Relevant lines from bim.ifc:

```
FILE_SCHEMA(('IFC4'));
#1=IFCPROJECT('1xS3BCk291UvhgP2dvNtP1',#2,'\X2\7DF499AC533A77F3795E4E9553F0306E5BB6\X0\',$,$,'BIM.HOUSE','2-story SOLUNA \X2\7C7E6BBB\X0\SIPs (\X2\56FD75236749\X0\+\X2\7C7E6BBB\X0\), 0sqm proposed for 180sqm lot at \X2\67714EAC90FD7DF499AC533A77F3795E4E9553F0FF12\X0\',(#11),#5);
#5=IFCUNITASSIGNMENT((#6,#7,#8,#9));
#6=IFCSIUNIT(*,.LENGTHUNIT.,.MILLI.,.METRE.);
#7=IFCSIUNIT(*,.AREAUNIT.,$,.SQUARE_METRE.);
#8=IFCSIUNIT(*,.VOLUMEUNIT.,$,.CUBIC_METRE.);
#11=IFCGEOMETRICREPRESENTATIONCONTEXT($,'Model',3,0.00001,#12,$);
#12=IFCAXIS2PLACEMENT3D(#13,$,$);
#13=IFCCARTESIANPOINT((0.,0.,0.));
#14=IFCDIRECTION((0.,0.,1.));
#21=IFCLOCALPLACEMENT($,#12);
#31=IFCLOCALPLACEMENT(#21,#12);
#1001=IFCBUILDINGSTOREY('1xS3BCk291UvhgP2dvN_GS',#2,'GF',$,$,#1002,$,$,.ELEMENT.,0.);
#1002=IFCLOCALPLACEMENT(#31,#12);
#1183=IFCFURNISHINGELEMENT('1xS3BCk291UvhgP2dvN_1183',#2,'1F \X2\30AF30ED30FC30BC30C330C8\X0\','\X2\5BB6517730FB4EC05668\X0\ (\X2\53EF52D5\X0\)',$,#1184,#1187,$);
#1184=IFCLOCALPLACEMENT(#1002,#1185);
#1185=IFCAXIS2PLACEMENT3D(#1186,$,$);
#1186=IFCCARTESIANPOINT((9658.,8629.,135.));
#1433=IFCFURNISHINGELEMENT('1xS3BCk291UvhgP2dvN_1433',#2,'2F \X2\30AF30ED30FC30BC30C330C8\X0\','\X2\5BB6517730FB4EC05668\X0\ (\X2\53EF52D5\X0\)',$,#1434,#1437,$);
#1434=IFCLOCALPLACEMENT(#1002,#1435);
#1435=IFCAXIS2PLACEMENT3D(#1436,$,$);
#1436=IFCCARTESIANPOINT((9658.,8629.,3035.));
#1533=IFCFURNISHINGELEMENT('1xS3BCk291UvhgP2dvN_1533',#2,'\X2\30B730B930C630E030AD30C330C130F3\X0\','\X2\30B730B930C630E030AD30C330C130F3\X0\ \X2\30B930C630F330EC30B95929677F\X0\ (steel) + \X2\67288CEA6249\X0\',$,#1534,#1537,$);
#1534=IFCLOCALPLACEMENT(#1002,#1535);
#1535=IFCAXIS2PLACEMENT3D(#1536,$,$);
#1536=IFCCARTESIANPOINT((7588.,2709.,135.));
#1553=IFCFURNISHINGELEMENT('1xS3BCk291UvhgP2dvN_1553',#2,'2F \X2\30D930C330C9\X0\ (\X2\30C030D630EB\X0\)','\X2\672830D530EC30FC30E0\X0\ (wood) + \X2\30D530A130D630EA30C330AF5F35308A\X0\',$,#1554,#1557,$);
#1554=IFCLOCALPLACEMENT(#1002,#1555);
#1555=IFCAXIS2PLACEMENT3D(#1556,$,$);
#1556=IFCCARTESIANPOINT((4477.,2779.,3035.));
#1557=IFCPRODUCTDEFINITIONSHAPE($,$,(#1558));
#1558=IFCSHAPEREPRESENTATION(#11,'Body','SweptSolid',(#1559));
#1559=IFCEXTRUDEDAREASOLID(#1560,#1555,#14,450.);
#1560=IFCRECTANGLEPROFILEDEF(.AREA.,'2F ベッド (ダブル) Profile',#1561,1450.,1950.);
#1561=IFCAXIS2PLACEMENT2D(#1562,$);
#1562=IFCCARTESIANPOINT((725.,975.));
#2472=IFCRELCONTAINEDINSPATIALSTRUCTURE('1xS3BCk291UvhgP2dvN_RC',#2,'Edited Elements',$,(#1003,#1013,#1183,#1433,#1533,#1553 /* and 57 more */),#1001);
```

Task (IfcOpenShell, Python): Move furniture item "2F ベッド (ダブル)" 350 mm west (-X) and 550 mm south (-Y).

```python
import ifcopenshell
import ifcopenshell.api.geometry
import ifcopenshell.util.placement

model = ifcopenshell.open("bim.ifc")

item = model.by_guid("1xS3BCk291UvhgP2dvN_1553")
matrix = ifcopenshell.util.placement.get_local_placement(item.ObjectPlacement)
matrix[0, 3] -= 350.0
matrix[1, 3] -= 550.0
ifcopenshell.api.geometry.edit_object_placement(model, product=item, matrix=matrix, is_si=False)

print(ifcopenshell.util.placement.get_local_placement(item.ObjectPlacement).round(3) + 0.0)

model.write("bim-out.ifc")
```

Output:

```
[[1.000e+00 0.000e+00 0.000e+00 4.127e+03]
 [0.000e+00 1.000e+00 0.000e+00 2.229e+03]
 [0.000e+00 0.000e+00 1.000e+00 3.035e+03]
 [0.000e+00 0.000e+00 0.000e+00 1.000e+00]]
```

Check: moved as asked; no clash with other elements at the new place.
